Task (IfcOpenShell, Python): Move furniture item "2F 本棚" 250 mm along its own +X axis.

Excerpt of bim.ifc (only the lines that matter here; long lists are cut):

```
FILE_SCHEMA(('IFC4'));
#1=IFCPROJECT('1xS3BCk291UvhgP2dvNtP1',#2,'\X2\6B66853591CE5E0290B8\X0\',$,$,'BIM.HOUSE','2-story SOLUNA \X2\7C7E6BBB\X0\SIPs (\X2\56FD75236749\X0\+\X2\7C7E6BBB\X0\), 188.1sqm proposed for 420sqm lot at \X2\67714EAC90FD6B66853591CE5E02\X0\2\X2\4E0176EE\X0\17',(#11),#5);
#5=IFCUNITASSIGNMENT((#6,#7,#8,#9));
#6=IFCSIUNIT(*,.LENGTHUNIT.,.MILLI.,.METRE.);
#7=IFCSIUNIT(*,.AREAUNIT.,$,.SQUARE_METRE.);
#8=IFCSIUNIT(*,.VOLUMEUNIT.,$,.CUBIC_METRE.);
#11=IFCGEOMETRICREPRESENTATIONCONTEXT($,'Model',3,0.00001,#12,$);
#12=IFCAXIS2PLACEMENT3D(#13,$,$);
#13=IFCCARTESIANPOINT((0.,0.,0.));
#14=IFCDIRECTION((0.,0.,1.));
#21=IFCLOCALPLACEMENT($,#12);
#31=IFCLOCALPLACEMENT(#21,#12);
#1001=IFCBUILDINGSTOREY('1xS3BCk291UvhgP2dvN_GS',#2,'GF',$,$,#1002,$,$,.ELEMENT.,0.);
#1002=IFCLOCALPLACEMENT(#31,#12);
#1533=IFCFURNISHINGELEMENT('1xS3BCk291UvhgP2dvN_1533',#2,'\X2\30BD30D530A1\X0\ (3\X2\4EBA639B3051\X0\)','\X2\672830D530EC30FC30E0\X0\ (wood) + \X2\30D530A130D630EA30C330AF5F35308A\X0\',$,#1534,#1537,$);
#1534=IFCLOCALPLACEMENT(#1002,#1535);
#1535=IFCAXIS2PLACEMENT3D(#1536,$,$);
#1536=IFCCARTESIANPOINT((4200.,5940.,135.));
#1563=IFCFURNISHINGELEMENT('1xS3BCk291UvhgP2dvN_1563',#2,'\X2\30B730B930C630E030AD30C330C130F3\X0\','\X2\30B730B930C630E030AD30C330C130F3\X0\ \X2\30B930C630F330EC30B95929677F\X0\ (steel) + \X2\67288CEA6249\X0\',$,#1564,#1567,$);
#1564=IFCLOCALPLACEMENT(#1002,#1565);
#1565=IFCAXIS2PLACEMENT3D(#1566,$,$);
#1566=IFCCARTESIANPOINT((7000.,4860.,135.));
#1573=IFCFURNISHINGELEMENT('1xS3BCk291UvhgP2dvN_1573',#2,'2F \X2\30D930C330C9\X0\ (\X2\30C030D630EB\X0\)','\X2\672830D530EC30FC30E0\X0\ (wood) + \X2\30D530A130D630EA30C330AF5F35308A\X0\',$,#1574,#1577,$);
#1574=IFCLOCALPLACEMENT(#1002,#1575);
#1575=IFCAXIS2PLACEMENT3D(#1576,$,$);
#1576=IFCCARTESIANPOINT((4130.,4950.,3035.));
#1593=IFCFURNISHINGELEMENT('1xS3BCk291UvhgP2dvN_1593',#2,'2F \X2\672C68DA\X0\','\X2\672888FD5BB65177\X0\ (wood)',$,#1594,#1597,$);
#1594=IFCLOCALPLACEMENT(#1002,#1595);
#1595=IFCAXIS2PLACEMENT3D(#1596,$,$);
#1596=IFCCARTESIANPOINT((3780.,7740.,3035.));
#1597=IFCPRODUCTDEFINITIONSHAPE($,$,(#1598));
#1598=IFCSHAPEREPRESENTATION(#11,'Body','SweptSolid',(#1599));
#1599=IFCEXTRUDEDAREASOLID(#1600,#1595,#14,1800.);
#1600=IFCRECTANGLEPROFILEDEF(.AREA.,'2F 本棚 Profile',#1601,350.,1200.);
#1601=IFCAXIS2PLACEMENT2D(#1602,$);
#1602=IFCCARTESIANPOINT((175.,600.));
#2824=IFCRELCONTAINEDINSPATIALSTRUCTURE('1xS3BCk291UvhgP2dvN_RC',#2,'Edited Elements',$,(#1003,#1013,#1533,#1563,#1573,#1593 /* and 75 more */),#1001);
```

```python
import ifcopenshell
import ifcopenshell.api.geometry
import ifcopenshell.util.placement

model = ifcopenshell.open("bim.ifc")

item = model.by_id(1593)
matrix = ifcopenshell.util.placement.get_local_placement(item.ObjectPlacement)
matrix[:3, 3] += matrix[:3, 0] * 250.0
ifcopenshell.api.geometry.edit_object_placement(model, product=item, matrix=matrix, is_si=False)

print(ifcopenshell.util.placement.get_local_placement(item.ObjectPlacement).round(3) + 0.0)

model.write("bim_v2.ifc")
```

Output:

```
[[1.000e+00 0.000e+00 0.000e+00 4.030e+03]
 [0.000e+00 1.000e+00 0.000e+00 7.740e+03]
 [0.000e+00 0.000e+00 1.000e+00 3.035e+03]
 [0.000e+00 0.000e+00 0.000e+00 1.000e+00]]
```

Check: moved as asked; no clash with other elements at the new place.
